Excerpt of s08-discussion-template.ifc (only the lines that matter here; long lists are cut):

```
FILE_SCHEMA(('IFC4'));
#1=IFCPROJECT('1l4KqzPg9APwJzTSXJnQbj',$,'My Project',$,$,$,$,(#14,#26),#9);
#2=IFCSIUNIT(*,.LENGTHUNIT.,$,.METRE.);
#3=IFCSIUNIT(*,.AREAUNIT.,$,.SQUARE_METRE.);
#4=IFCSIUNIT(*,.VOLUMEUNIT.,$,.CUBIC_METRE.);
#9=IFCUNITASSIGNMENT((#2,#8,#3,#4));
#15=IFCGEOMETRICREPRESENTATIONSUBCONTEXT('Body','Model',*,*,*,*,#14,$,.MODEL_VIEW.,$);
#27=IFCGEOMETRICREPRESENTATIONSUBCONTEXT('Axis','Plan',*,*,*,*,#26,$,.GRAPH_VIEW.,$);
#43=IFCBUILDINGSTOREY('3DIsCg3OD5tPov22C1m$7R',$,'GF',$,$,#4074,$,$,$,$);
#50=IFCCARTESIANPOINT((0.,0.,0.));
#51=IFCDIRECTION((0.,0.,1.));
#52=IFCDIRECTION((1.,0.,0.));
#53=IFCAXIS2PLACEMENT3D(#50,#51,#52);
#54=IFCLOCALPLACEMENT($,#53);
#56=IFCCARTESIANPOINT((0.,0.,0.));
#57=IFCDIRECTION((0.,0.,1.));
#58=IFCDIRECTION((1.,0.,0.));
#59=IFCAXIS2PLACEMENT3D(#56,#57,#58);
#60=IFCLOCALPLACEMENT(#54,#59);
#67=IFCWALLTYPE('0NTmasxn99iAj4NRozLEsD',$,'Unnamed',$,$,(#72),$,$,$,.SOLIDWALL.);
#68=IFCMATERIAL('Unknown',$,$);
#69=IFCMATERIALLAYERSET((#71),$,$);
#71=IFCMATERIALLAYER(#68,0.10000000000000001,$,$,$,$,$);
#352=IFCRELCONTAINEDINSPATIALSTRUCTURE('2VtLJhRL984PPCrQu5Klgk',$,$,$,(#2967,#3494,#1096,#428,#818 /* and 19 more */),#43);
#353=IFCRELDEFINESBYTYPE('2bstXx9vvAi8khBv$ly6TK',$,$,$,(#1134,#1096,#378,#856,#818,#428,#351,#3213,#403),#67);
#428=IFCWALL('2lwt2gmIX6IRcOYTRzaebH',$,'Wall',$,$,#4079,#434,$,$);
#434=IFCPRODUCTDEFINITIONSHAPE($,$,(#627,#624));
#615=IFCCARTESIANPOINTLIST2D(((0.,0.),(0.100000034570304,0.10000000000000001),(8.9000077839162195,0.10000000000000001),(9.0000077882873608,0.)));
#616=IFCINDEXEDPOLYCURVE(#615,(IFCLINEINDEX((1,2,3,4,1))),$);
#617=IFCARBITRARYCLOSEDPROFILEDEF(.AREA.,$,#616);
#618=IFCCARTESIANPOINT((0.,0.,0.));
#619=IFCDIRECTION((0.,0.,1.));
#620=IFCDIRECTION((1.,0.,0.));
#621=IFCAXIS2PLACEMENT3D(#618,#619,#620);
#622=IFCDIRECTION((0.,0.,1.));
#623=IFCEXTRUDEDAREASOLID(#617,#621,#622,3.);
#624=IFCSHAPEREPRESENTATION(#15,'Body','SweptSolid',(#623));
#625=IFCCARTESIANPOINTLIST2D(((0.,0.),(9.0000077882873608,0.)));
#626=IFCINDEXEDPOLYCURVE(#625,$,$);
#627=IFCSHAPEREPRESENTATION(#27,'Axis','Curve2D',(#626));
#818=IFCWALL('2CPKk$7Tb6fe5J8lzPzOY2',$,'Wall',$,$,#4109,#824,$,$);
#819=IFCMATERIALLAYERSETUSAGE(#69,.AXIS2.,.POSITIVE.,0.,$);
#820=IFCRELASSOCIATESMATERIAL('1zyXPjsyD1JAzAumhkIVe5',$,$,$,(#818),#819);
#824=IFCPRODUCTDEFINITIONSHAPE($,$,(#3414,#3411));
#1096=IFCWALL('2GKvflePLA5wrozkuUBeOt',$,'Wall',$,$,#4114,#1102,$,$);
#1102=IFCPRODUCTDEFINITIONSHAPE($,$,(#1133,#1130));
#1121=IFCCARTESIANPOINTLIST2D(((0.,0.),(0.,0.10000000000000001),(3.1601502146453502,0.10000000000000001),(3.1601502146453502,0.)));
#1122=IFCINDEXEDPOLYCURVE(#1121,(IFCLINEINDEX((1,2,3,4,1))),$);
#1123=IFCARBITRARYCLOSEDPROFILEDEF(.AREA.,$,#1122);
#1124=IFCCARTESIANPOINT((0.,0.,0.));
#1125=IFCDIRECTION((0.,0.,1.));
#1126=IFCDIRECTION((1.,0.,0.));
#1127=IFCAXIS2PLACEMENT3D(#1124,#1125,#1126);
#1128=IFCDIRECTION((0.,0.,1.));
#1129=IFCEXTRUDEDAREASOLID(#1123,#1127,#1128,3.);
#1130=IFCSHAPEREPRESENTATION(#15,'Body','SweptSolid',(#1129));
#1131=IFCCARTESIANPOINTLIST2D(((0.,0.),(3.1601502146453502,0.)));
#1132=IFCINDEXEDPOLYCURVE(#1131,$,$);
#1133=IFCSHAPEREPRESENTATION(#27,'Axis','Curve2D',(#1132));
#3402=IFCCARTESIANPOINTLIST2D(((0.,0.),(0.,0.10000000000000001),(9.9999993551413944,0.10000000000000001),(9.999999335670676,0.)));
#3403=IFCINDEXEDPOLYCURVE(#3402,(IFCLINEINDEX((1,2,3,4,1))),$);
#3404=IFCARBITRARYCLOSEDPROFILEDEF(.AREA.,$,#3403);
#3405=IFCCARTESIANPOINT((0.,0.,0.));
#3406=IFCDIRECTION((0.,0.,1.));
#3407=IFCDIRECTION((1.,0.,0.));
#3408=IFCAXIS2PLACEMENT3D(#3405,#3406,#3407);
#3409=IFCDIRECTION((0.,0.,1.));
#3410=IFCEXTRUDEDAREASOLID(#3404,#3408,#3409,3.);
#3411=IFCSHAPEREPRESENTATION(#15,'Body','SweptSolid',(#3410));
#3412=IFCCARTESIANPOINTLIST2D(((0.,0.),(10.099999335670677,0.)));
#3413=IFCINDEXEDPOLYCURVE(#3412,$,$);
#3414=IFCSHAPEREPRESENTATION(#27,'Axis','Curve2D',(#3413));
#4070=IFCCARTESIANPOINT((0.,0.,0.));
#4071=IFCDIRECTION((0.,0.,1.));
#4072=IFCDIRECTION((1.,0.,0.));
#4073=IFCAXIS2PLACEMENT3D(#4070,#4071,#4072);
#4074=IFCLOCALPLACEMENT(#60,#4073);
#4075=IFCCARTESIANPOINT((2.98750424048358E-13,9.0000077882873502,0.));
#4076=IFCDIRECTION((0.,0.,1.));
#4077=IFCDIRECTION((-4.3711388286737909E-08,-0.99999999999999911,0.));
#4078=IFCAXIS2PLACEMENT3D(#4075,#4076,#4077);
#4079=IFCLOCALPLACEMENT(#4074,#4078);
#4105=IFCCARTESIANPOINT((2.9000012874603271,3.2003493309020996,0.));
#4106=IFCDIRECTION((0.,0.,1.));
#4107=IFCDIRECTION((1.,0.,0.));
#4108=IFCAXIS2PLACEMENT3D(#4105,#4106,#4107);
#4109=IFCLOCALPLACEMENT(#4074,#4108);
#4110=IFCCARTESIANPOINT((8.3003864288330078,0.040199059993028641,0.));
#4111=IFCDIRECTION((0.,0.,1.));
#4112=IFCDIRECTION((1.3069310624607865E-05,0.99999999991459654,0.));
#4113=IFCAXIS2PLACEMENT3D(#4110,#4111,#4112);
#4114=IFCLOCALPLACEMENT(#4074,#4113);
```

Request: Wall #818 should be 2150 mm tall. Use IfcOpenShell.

```python
import ifcopenshell
import ifcopenshell.geom
import ifcopenshell.util.representation
import ifcopenshell.util.shape

model = ifcopenshell.open("s08-discussion-template.ifc")
settings = ifcopenshell.geom.settings()


def volume(element):
    """Net volume in cubic metres, openings subtracted."""
    shape = ifcopenshell.geom.create_shape(settings, element)
    return ifcopenshell.util.shape.get_volume(shape.geometry)


wall = model.by_guid("2CPKk$7Tb6fe5J8lzPzOY2")
before = volume(wall)

body = ifcopenshell.util.representation.get_representation(wall, "Model", "Body")
solid = body.Items[0]
old_height = solid.Depth
solid.Depth = 2.15
after = volume(wall)

print(f"height {old_height:g} -> {solid.Depth:g}, volume {before:.3f} -> {after:.3f} m3")

model.write("s08-discussion-template_v2.ifc")
```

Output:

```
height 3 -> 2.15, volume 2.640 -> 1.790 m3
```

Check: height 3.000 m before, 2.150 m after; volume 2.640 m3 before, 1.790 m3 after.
